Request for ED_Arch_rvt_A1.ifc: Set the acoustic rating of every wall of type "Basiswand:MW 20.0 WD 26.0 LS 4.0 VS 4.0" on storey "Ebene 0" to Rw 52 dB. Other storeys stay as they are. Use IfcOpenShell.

First a look at what the model holds.

```python
import ifcopenshell
import ifcopenshell.util.element

model = ifcopenshell.open("ED_Arch_rvt_A1.ifc")
print(model.schema)
storey = next(s for s in model.by_type("IfcBuildingStorey") if s.Name == "Ebene 0")
walls = [e for e in ifcopenshell.util.element.get_decomposition(storey) if e.is_a("IfcWall")]
seen = {}
for e in walls:
    element_type = ifcopenshell.util.element.get_type(e)
    key = (element_type.Name if element_type != e and element_type else None, ifcopenshell.util.element.get_pset(e, "Pset_WallCommon", "AcousticRating"))
    seen[key] = seen.get(key, 0) + 1
for (name, value), count in sorted(seen.items(), key=str):
    print(count, "x", name, "|", value)
```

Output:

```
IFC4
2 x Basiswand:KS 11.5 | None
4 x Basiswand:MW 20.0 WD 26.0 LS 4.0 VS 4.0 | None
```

```python
import ifcopenshell
import ifcopenshell.api.pset
import ifcopenshell.util.element

model = ifcopenshell.open("ED_Arch_rvt_A1.ifc")

storey = next(s for s in model.by_type("IfcBuildingStorey") if s.Name == "Ebene 0")
walls = [e for e in ifcopenshell.util.element.get_decomposition(storey) if e.is_a("IfcWall")]

count = 0
for e in walls:
    element_type = ifcopenshell.util.element.get_type(e)
    if element_type in (None, e) or element_type.Name != "Basiswand:MW 20.0 WD 26.0 LS 4.0 VS 4.0":
        continue
    # add_pset returns the element's existing set when there is one.
    pset = ifcopenshell.api.pset.add_pset(model, product=e, name="Pset_WallCommon")
    ifcopenshell.api.pset.edit_pset(model, pset=pset, properties={"AcousticRating": "Rw 52 dB"})
    count += 1

print(count, "walls updated")

model.write("ED_Arch_rvt_A1_edited.ifc")
```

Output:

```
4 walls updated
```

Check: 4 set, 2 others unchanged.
